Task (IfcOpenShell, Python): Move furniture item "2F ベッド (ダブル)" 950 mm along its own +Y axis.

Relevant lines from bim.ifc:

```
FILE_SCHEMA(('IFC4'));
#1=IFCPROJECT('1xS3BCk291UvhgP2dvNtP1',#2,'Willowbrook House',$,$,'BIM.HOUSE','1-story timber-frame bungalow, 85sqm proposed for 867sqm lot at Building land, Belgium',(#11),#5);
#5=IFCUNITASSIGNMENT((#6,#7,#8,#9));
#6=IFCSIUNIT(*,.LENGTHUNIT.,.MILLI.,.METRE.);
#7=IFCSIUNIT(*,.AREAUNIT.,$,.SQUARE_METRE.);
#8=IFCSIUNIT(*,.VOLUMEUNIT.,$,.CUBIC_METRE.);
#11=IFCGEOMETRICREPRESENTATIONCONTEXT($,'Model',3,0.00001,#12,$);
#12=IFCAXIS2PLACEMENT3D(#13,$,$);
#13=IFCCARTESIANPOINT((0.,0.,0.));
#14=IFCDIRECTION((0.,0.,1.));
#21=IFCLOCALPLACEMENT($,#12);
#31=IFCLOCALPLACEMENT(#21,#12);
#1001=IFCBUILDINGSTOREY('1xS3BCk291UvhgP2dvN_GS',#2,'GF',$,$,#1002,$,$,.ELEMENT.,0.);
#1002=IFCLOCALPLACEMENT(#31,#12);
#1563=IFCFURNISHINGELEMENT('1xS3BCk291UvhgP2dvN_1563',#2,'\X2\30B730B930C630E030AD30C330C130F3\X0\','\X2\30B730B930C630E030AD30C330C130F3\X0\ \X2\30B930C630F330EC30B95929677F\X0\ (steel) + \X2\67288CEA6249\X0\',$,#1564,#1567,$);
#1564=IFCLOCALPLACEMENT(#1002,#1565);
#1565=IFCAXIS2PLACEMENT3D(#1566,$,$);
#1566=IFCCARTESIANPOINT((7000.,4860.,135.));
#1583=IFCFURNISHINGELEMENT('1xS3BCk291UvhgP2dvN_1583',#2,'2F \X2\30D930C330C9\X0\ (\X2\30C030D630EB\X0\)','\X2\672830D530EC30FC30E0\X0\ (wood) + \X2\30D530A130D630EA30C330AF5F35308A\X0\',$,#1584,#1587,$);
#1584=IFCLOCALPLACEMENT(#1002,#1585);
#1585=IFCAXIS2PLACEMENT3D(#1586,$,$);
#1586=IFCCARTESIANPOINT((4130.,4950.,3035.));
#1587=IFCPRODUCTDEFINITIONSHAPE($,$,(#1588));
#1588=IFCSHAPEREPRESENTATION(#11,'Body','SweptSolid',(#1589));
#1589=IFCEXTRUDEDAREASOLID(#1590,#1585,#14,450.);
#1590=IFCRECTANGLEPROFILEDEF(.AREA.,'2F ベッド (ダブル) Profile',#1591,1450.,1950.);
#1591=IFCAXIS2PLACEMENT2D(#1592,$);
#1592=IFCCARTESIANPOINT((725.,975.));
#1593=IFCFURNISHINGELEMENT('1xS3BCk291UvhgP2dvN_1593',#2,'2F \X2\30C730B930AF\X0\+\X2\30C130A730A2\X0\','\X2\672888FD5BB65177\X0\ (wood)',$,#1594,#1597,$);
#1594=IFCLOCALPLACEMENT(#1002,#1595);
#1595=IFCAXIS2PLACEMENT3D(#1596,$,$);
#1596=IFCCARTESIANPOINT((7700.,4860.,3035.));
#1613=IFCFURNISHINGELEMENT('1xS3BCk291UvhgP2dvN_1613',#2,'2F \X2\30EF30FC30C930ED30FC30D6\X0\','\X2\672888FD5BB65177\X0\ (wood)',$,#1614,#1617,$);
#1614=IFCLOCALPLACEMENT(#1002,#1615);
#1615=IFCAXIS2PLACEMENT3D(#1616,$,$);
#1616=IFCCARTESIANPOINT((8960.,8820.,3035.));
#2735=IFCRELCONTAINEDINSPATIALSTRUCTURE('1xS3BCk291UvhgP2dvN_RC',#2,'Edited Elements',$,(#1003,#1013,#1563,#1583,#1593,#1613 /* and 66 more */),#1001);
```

```python
import ifcopenshell
import ifcopenshell.api.geometry
import ifcopenshell.util.placement
import ifcopenshell.util.unit

model = ifcopenshell.open("bim.ifc")
unit_scale = ifcopenshell.util.unit.calculate_unit_scale(model)

item = model.by_guid("1xS3BCk291UvhgP2dvN_1583")
matrix = ifcopenshell.util.placement.get_local_placement(item.ObjectPlacement)
matrix[:3, 3] += matrix[:3, 1] * 0.95 / unit_scale
ifcopenshell.api.geometry.edit_object_placement(model, product=item, matrix=matrix, is_si=False)

print(ifcopenshell.util.placement.get_local_placement(item.ObjectPlacement).round(3) + 0.0)

model.write("bim_rev.ifc")
```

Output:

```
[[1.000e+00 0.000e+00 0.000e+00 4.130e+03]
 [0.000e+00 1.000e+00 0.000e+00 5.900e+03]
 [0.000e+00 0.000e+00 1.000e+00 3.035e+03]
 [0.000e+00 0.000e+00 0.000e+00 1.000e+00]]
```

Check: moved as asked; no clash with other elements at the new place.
